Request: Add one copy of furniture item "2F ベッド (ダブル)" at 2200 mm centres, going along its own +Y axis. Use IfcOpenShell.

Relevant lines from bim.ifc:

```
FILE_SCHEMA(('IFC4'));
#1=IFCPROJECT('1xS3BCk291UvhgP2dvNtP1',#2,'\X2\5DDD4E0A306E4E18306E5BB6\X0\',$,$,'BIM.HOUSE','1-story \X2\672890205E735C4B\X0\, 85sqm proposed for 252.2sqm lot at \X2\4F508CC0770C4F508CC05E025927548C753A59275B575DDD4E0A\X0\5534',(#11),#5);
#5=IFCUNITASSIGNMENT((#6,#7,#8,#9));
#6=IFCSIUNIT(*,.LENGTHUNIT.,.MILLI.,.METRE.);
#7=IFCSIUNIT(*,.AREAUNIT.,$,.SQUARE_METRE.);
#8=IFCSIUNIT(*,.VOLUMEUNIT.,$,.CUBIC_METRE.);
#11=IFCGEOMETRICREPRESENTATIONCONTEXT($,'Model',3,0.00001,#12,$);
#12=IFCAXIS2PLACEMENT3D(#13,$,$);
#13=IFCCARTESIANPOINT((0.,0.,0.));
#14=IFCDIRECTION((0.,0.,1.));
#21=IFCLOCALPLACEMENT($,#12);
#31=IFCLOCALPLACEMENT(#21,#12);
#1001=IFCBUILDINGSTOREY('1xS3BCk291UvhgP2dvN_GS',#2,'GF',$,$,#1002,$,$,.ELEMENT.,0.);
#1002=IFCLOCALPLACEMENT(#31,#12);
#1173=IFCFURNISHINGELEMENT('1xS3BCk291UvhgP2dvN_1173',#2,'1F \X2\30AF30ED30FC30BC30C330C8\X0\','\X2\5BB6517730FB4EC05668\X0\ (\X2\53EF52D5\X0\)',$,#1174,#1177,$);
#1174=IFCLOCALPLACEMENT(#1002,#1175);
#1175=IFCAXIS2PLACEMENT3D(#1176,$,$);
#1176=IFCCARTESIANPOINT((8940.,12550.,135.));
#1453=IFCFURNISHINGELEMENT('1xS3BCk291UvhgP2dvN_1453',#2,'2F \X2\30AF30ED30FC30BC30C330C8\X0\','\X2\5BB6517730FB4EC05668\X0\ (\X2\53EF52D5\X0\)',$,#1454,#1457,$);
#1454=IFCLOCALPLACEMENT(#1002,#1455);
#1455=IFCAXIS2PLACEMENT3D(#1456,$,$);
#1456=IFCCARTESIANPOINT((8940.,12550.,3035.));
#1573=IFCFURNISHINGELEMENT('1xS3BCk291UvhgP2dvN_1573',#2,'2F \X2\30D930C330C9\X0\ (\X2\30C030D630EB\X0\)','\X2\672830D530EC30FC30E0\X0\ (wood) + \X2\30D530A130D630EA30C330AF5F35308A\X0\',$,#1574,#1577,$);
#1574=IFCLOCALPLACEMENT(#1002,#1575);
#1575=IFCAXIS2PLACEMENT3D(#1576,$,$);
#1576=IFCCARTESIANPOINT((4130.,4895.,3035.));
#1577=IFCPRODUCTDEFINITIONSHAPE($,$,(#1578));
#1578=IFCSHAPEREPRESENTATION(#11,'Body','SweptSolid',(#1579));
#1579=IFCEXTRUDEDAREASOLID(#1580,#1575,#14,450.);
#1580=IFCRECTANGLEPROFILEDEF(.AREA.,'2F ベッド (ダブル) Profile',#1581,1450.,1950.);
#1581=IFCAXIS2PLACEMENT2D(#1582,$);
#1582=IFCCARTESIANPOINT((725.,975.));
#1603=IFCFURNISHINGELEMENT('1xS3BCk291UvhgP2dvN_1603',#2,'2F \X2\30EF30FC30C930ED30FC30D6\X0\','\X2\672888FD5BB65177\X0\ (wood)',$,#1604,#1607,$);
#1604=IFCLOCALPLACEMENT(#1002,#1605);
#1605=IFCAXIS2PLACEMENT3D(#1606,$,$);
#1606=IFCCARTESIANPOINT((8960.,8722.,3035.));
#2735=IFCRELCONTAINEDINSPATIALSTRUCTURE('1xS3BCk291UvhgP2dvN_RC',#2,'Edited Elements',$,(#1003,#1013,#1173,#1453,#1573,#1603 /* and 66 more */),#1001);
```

```python
import ifcopenshell
import ifcopenshell.api.geometry
import ifcopenshell.api.root
import ifcopenshell.util.element
import ifcopenshell.util.placement
import ifcopenshell.util.unit

model = ifcopenshell.open("bim.ifc")
unit_scale = ifcopenshell.util.unit.calculate_unit_scale(model)


def reuse_history(source, copy):
    """copy_class also copies each property set's owner history, people and application; keep the originals."""
    for rel in copy.IsDefinedBy:
        if rel.is_a("IfcRelDefinesByProperties") and (history := rel.RelatingPropertyDefinition.OwnerHistory):
            rel.RelatingPropertyDefinition.OwnerHistory = source.OwnerHistory
            ifcopenshell.util.element.remove_deep2(model, history)


source = model.by_guid("1xS3BCk291UvhgP2dvN_1573")
base = ifcopenshell.util.placement.get_local_placement(source.ObjectPlacement)
step = base[:3, 1] * 2.2 / unit_scale

for i in range(1, 2):
    copy = ifcopenshell.api.root.copy_class(model, product=source)
    copy.Representation = ifcopenshell.util.element.copy_deep(
        model, source.Representation, exclude=["IfcGeometricRepresentationContext", "IfcRepresentationMap"]
    )
    reuse_history(source, copy)
    matrix = base.copy()
    matrix[:3, 3] += i * step
    print("added at", matrix[:3, 3].round(3) + 0.0)
    ifcopenshell.api.geometry.edit_object_placement(model, product=copy, matrix=matrix, is_si=False)

model.write("bim_rev.ifc")
```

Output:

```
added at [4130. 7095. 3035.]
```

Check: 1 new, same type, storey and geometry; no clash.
